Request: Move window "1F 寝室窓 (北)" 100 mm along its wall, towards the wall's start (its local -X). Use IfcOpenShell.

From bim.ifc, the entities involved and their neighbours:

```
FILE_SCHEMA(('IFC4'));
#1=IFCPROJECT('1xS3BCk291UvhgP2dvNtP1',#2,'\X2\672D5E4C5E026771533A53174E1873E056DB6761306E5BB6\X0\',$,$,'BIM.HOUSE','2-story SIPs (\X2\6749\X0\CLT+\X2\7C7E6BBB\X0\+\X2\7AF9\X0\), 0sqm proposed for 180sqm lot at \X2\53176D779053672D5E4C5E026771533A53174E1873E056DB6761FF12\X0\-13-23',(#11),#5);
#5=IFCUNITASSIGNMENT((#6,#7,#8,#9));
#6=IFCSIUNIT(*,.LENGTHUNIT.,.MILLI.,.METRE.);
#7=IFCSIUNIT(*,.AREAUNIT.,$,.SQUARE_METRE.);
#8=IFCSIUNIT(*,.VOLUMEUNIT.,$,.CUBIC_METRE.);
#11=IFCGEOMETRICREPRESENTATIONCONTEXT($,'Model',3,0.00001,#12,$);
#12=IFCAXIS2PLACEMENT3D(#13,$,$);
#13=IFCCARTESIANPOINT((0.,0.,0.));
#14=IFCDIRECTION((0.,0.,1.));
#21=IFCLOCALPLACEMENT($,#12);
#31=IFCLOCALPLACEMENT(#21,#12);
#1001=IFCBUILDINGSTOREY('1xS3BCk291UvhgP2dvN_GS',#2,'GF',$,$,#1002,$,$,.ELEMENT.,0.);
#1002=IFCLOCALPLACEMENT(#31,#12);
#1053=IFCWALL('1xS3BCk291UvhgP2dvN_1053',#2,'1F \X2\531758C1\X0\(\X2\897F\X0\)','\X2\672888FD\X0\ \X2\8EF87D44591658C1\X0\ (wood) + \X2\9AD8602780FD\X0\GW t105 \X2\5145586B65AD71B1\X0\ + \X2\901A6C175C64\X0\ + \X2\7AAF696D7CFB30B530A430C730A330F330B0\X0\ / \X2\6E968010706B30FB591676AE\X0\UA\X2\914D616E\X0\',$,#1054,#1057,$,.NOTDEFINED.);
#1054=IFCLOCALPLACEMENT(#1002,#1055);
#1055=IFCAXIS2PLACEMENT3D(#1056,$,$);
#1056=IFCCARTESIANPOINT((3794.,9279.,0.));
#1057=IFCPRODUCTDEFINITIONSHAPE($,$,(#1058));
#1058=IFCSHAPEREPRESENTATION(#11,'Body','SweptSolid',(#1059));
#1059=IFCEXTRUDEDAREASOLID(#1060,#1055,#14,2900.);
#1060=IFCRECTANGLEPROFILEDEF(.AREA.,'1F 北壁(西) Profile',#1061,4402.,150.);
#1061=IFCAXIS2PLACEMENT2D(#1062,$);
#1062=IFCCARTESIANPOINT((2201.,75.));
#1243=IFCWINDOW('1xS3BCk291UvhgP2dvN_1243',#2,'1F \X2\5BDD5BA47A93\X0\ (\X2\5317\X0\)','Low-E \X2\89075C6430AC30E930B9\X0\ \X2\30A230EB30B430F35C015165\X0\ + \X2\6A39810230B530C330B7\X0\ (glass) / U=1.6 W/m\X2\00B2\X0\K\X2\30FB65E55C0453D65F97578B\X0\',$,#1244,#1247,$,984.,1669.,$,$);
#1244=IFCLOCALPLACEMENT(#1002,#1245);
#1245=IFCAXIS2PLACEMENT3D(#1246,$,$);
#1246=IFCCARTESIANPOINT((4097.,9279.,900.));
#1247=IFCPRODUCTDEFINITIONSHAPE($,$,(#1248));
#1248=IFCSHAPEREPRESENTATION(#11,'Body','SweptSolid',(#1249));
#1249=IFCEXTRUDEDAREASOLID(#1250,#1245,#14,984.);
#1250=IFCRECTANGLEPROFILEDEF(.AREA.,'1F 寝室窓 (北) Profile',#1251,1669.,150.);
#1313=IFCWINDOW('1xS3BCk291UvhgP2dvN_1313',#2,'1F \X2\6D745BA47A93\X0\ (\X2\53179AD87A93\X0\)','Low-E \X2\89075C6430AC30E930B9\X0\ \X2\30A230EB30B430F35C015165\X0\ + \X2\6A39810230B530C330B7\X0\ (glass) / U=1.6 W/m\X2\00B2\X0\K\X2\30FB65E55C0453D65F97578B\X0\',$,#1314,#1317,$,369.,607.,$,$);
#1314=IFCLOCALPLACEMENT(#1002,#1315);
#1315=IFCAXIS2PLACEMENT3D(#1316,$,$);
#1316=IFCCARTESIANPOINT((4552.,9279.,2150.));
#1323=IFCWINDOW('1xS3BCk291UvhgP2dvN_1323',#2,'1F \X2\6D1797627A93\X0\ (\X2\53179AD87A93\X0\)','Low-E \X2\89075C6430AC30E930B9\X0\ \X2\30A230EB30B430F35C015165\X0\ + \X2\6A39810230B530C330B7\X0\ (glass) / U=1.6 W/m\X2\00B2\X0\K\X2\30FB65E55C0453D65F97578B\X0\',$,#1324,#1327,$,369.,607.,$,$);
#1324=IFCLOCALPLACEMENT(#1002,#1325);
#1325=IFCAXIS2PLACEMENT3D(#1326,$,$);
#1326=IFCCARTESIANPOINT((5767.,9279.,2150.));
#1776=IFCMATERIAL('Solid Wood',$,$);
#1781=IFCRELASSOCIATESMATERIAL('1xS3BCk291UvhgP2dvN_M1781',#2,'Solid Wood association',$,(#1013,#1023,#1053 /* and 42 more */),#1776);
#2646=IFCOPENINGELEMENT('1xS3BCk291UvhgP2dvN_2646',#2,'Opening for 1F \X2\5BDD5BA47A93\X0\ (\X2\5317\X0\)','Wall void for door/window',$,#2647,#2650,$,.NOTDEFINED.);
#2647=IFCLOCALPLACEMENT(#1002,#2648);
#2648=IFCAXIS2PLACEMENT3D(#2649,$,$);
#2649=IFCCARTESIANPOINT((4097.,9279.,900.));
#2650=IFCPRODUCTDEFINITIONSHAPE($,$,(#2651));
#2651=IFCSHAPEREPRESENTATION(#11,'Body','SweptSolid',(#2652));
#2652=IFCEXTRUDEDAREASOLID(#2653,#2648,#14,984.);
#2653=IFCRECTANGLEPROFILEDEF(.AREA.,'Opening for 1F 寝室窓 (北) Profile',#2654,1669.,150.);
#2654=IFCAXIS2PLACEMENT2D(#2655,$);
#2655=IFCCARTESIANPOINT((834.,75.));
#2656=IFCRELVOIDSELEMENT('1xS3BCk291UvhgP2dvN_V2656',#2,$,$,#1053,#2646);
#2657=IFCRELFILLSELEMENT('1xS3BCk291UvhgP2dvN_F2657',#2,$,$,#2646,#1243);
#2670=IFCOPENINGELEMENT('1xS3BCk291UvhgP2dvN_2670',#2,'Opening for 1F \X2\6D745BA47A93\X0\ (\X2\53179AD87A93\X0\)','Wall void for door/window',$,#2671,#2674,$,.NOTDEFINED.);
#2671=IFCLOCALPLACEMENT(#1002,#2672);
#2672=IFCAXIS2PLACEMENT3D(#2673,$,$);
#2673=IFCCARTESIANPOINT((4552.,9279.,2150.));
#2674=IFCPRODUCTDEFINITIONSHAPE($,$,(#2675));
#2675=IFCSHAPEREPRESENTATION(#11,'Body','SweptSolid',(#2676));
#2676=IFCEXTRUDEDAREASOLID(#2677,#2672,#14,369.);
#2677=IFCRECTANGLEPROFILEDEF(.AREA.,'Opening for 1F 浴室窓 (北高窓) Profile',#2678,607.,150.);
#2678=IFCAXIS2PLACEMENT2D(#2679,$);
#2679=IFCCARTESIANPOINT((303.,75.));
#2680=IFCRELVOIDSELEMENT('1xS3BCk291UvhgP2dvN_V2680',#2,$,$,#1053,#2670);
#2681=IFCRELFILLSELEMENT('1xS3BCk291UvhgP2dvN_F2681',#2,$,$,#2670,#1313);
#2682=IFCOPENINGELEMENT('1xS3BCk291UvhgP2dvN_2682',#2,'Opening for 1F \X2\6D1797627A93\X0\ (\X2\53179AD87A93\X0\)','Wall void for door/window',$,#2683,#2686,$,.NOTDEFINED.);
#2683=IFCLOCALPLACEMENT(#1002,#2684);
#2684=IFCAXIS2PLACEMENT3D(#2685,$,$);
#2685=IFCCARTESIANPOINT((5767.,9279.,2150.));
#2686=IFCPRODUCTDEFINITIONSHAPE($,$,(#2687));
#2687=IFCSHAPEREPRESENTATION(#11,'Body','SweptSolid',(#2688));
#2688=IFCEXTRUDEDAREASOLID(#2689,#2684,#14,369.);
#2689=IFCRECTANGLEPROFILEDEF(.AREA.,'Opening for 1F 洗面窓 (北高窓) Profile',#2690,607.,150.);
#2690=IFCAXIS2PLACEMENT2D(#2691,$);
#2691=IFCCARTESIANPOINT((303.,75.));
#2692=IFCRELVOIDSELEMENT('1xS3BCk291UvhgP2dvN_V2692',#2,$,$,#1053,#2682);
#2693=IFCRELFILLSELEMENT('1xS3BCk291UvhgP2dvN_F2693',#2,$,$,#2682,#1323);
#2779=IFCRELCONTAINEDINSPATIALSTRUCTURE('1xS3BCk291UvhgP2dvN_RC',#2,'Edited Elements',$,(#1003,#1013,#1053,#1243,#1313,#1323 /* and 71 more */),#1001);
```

```python
import ifcopenshell
import ifcopenshell.api.geometry
import ifcopenshell.util.placement

model = ifcopenshell.open("bim.ifc")

window = model.by_guid("1xS3BCk291UvhgP2dvN_1243")
opening = window.FillsVoids[0].RelatingOpeningElement
wall = opening.VoidsElements[0].RelatingBuildingElement

wall_matrix = ifcopenshell.util.placement.get_local_placement(wall.ObjectPlacement)
shift = wall_matrix[:3, 0] * -100.0
before = ifcopenshell.util.placement.get_local_placement(window.ObjectPlacement)[:3, 3].copy()

# The window is not placed relative to its opening, so move both.
for product in (opening, window):
    matrix = ifcopenshell.util.placement.get_local_placement(product.ObjectPlacement)
    matrix[:3, 3] += shift
    ifcopenshell.api.geometry.edit_object_placement(model, product=product, matrix=matrix, is_si=False)

after = ifcopenshell.util.placement.get_local_placement(window.ObjectPlacement)[:3, 3]
print("window moved by", (after - before).round(3) + 0.0)

model.write("bim-out.ifc")
```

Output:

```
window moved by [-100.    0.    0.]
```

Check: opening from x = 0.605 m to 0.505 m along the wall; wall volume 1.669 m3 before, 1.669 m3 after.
